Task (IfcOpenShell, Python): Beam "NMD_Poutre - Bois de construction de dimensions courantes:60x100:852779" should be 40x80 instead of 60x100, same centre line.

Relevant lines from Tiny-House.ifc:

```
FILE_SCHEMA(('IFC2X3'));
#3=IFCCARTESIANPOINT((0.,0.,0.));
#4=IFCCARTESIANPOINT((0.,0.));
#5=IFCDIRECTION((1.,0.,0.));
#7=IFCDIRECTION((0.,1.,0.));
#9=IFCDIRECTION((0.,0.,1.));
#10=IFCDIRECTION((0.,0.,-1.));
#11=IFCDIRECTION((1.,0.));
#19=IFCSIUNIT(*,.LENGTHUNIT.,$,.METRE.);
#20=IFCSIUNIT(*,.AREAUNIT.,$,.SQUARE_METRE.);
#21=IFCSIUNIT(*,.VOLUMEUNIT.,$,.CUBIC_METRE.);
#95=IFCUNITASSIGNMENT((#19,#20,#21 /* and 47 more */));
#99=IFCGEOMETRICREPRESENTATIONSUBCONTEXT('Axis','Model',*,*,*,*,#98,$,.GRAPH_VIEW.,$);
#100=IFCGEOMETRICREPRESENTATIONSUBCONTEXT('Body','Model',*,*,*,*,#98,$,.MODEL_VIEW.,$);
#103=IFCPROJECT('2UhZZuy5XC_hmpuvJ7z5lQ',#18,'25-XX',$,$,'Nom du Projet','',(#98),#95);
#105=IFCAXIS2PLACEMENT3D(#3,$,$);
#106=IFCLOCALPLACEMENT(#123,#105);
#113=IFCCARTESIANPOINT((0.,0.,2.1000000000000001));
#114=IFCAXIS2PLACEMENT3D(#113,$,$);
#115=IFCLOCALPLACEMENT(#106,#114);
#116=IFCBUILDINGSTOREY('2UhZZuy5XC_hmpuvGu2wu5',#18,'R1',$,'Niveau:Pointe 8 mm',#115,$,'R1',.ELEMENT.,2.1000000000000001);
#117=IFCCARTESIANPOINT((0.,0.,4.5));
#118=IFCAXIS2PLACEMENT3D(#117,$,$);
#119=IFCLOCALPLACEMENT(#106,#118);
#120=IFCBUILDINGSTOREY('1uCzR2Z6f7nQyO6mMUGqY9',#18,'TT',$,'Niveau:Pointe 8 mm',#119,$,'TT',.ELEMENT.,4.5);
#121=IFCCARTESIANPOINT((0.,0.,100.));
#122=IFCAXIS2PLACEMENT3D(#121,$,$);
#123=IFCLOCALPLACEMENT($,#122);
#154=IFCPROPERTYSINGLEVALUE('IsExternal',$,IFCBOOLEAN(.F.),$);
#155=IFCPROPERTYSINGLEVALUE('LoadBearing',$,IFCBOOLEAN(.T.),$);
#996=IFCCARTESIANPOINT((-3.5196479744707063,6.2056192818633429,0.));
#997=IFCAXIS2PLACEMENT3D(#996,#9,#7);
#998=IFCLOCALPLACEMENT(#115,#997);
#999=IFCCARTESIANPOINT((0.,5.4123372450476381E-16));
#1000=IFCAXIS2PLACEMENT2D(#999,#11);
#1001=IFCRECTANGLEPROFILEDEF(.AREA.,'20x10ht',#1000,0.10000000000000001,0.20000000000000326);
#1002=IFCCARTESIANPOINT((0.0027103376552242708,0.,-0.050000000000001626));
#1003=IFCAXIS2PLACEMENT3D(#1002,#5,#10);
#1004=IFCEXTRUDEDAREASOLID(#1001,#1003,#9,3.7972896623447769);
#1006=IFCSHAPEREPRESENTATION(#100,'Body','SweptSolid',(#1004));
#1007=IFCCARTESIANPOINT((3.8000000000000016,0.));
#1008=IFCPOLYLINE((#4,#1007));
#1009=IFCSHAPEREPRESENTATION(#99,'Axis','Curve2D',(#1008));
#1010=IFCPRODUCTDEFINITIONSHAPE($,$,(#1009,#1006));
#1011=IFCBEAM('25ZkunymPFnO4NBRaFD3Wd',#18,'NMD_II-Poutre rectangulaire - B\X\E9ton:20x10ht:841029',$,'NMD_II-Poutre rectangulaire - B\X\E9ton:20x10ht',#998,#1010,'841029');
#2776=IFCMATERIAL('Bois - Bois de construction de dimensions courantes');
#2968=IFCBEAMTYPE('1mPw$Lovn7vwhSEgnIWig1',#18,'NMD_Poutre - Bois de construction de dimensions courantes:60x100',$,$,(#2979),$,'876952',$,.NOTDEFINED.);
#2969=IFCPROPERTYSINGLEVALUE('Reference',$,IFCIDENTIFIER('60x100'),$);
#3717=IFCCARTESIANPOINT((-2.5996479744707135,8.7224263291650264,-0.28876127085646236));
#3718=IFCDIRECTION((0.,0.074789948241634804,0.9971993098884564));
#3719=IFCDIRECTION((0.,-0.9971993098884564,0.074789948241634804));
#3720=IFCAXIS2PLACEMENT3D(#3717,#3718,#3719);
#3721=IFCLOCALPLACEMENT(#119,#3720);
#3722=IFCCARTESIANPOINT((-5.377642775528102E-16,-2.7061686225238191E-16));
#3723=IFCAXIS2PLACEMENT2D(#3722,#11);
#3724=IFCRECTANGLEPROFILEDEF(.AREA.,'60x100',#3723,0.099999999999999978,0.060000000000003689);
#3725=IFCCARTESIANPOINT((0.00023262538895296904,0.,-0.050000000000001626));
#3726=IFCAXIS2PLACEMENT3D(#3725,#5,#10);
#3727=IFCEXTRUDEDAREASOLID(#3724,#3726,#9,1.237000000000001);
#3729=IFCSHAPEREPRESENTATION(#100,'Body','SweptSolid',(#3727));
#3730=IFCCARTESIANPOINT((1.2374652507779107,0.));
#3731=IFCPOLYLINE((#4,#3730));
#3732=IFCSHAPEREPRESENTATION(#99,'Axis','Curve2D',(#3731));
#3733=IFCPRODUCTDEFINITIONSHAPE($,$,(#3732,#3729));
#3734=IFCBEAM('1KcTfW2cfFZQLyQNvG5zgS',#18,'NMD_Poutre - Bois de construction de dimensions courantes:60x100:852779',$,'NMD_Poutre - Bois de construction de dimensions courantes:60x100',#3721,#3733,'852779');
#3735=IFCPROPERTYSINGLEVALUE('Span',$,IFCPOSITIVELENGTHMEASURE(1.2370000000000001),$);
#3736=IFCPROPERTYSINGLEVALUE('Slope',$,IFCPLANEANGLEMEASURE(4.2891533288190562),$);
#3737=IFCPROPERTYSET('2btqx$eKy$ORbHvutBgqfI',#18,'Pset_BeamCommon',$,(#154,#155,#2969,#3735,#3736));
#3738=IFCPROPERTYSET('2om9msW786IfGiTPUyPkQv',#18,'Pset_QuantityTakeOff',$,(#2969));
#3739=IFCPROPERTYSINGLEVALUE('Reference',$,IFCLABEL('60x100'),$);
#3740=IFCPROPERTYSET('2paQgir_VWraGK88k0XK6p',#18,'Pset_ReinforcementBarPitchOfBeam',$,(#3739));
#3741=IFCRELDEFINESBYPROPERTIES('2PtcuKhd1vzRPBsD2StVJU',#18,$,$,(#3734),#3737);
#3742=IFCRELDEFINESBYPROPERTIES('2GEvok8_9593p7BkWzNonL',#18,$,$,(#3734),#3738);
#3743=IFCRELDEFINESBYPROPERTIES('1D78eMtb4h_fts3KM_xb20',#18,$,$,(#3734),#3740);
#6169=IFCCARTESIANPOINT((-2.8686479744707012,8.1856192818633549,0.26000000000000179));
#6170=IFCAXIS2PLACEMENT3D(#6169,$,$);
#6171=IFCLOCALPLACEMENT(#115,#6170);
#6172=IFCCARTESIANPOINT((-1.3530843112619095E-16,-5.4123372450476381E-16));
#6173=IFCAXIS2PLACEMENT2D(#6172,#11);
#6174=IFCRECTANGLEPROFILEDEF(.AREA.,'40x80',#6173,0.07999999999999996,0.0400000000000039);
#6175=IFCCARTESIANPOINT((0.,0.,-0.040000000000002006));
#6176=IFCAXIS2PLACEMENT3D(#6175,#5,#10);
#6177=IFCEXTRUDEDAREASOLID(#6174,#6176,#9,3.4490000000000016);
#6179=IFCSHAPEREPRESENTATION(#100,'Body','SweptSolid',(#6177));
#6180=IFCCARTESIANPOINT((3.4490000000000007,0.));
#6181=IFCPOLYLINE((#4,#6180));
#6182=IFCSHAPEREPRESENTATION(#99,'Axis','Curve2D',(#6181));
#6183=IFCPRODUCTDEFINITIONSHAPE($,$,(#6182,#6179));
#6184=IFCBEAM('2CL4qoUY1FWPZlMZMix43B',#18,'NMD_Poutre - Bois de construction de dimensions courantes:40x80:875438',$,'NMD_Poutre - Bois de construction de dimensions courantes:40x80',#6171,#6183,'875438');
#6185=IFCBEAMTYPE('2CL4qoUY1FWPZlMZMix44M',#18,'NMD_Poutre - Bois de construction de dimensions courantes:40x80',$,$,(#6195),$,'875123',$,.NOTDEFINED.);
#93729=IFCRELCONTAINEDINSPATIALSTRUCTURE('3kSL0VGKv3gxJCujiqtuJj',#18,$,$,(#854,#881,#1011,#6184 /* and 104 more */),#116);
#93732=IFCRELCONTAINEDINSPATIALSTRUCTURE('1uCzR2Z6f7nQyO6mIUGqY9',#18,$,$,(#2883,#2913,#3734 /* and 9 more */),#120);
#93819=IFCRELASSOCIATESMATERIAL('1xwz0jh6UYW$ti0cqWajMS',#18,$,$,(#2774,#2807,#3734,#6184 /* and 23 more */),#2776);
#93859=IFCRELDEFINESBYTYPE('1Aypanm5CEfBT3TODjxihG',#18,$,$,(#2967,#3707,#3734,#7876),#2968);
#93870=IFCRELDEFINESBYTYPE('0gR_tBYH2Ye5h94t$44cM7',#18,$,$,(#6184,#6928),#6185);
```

```python
import ifcopenshell
import ifcopenshell.api.pset
import ifcopenshell.api.type
import ifcopenshell.util.element
import ifcopenshell.util.representation

model = ifcopenshell.open("Tiny-House.ifc")

member = model.by_guid("1KcTfW2cfFZQLyQNvG5zgS")
source = next(p for p in model.by_type("IfcRectangleProfileDef") if p.ProfileName == "40x80")

body = ifcopenshell.util.representation.get_representation(member, "Model", "Body")
solid = body.Items[0]
old_profile = solid.SweptArea

# Copy the section's sizes but keep this member's own profile position.
profile = ifcopenshell.util.element.copy(model, source)
profile.Position = old_profile.Position
solid.SweptArea = profile
if not model.get_total_inverses(old_profile):
    ifcopenshell.util.element.remove_deep2(model, old_profile)

new_type = model.by_id(6185)
ifcopenshell.api.type.assign_type(
    model, related_objects=[member], relating_type=new_type, should_map_representations=False
)
member.Name = member.Name.replace("60x100", "40x80")
member.ObjectType = "NMD_Poutre - Bois de construction de dimensions courantes:40x80"
pset = model.by_id(ifcopenshell.util.element.get_pset(member, "Pset_BeamCommon", should_inherit=False)["id"])
ifcopenshell.api.pset.edit_pset(model, pset=pset, properties={"Reference": "40x80"})
pset = model.by_id(ifcopenshell.util.element.get_pset(member, "Pset_QuantityTakeOff", should_inherit=False)["id"])
ifcopenshell.api.pset.edit_pset(model, pset=pset, properties={"Reference": "40x80"})
pset = model.by_id(ifcopenshell.util.element.get_pset(member, "Pset_ReinforcementBarPitchOfBeam", should_inherit=False)["id"])
ifcopenshell.api.pset.edit_pset(model, pset=pset, properties={"Reference": "40x80"})

print(solid.SweptArea)

model.write("Tiny-House_edited.ifc")
```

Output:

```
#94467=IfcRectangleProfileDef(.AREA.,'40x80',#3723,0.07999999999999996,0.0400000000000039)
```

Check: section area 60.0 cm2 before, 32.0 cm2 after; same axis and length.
